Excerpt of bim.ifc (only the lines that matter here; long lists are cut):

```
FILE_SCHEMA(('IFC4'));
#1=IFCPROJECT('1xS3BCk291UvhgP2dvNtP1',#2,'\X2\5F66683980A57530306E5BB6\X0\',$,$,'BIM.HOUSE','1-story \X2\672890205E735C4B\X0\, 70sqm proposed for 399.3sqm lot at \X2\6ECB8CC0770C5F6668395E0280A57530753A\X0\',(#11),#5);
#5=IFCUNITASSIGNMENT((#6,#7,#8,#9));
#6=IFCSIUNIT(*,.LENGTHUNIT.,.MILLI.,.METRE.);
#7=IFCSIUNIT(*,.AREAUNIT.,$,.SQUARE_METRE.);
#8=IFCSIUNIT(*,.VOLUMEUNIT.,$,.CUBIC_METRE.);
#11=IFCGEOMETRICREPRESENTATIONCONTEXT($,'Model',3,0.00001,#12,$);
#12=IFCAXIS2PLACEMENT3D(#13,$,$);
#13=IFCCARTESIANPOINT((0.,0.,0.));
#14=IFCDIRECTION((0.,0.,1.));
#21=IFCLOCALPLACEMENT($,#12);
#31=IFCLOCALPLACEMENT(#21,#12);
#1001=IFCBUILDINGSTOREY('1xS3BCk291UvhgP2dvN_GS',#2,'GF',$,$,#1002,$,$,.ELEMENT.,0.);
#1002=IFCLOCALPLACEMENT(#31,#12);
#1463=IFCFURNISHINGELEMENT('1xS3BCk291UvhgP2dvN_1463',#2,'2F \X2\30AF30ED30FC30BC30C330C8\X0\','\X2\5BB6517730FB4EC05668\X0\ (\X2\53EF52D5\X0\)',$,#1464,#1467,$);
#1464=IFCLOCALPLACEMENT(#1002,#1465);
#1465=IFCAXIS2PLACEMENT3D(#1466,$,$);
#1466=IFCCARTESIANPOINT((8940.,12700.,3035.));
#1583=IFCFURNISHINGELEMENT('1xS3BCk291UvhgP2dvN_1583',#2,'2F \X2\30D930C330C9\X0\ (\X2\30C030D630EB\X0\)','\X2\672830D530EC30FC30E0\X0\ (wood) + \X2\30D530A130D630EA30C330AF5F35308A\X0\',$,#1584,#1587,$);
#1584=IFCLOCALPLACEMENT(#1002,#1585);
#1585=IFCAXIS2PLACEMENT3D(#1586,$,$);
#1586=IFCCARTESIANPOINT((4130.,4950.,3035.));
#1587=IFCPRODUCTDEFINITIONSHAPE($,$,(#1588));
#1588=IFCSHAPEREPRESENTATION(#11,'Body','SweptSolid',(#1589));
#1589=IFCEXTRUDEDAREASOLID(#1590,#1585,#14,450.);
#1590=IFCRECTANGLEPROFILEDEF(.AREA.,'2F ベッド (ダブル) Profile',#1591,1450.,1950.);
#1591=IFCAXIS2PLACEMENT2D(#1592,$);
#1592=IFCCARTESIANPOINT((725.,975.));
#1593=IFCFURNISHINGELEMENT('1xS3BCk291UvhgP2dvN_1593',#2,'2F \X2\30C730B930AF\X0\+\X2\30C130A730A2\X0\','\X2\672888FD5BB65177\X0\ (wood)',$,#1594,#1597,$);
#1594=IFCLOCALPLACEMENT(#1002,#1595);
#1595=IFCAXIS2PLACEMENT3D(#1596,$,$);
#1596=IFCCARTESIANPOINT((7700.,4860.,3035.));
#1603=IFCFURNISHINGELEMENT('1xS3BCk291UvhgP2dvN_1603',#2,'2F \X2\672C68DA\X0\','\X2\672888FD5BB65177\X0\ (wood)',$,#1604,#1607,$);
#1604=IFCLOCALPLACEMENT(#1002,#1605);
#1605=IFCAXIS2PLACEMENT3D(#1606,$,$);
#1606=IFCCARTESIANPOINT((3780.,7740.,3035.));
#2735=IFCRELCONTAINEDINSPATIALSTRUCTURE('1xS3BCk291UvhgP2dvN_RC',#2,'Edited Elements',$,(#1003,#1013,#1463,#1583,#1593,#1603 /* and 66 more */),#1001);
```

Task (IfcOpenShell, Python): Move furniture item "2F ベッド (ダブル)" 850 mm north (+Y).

```python
import ifcopenshell
import ifcopenshell.api.geometry
import ifcopenshell.util.placement

model = ifcopenshell.open("bim.ifc")

item = model.by_id(1583)
matrix = ifcopenshell.util.placement.get_local_placement(item.ObjectPlacement)
matrix[1, 3] += 850.0
ifcopenshell.api.geometry.edit_object_placement(model, product=item, matrix=matrix, is_si=False)

print(ifcopenshell.util.placement.get_local_placement(item.ObjectPlacement).round(3) + 0.0)

model.write("bim_edited.ifc")
```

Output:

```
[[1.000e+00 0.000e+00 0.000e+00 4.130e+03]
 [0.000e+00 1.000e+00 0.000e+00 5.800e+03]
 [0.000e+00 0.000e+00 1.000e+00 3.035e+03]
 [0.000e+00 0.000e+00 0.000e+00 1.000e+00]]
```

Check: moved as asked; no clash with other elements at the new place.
